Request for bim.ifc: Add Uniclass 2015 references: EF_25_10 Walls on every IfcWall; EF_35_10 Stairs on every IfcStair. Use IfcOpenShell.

First a look at what the model holds.

```python
import ifcopenshell

model = ifcopenshell.open("bim.ifc")
print(model.schema)
print("classifications:", [c.Name for c in model.by_type("IfcClassification")])
for ifc_class in ("IfcDoor", "IfcRoof", "IfcStair", "IfcWall", "IfcWindow"):
    print(ifc_class, len(model.by_type(ifc_class)))
```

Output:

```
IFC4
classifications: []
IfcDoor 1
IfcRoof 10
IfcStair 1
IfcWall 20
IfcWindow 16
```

```python
import ifcopenshell
import ifcopenshell.api.classification

model = ifcopenshell.open("bim.ifc")

system = ifcopenshell.api.classification.add_classification(model, classification="Uniclass 2015")

codes = {
    "IfcWall": ("EF_25_10", "Walls"),
    "IfcStair": ("EF_35_10", "Stairs"),
}
for ifc_class, (code, name) in codes.items():
    products = model.by_type(ifc_class)
    ifcopenshell.api.classification.add_reference(
        model, products=products, classification=system, identification=code, name=name
    )
    print(code, len(products))

model.write("bim-out.ifc")
```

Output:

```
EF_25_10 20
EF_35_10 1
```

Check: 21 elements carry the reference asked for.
